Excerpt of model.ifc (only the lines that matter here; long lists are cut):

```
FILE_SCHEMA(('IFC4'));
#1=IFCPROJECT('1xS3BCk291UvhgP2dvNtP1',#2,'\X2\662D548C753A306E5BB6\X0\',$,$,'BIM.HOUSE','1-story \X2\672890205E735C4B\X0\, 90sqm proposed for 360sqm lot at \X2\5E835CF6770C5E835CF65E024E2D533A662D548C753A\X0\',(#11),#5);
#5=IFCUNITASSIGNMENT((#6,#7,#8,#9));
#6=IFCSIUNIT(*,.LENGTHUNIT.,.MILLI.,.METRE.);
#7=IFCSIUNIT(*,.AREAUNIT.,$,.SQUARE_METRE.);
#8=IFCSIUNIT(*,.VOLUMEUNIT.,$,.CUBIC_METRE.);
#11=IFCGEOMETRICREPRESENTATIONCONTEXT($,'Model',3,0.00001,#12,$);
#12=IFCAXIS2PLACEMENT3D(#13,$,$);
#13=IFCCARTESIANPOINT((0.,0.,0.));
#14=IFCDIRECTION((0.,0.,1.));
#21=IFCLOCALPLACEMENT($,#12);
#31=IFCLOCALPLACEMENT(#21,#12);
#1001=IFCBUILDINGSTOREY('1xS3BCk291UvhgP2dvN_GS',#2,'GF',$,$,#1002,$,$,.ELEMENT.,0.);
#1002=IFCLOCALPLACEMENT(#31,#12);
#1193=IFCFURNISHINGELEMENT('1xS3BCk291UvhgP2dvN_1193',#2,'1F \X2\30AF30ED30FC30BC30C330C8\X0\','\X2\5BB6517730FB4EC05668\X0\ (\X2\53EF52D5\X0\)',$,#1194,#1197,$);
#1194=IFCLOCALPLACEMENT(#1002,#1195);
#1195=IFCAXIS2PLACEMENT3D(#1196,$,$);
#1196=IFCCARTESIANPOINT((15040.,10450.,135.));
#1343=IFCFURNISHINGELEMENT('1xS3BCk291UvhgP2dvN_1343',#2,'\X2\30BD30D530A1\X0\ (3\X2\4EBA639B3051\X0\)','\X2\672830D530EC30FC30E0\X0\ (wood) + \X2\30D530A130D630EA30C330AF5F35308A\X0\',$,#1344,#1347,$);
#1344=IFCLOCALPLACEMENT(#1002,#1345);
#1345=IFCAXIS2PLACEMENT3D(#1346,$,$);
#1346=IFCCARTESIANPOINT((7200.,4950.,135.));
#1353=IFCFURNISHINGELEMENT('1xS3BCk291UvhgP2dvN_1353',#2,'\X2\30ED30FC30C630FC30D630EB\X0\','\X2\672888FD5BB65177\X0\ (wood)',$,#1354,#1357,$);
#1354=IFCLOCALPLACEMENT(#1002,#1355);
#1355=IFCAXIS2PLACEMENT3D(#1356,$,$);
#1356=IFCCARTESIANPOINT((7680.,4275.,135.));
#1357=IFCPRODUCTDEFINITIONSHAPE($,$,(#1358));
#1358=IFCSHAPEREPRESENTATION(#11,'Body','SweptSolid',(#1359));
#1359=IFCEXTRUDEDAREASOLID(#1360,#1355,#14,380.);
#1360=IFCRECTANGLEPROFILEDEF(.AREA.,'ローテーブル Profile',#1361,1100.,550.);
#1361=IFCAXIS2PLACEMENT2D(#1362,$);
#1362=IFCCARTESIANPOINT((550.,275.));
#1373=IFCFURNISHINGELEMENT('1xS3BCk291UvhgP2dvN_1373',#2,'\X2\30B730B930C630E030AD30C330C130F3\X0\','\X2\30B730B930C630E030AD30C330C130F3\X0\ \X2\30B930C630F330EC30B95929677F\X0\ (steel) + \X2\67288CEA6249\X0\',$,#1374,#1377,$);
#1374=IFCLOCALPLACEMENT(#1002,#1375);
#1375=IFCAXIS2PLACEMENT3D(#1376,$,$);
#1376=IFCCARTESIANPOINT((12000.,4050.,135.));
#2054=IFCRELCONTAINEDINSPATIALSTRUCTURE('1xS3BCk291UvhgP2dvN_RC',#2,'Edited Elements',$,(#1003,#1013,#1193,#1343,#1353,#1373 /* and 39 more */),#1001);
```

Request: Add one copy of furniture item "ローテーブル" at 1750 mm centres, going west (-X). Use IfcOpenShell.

```python
import numpy as np
import ifcopenshell
import ifcopenshell.api.geometry
import ifcopenshell.api.root
import ifcopenshell.util.element
import ifcopenshell.util.placement
import ifcopenshell.util.unit

model = ifcopenshell.open("model.ifc")
unit_scale = ifcopenshell.util.unit.calculate_unit_scale(model)


def reuse_history(source, copy):
    """copy_class also copies each property set's owner history, people and application; keep the originals."""
    for rel in copy.IsDefinedBy:
        if rel.is_a("IfcRelDefinesByProperties") and (history := rel.RelatingPropertyDefinition.OwnerHistory):
            rel.RelatingPropertyDefinition.OwnerHistory = source.OwnerHistory
            ifcopenshell.util.element.remove_deep2(model, history)


source = model.by_guid("1xS3BCk291UvhgP2dvN_1353")
base = ifcopenshell.util.placement.get_local_placement(source.ObjectPlacement)
step = np.array([-1.0, 0.0, 0.0]) * 1.75 / unit_scale

for i in range(1, 2):
    copy = ifcopenshell.api.root.copy_class(model, product=source)
    copy.Representation = ifcopenshell.util.element.copy_deep(
        model, source.Representation, exclude=["IfcGeometricRepresentationContext", "IfcRepresentationMap"]
    )
    reuse_history(source, copy)
    matrix = base.copy()
    matrix[:3, 3] += i * step
    print("added at", matrix[:3, 3].round(3) + 0.0)
    ifcopenshell.api.geometry.edit_object_placement(model, product=copy, matrix=matrix, is_si=False)

model.write("model_v2.ifc")
```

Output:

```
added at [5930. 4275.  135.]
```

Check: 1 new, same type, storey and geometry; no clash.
